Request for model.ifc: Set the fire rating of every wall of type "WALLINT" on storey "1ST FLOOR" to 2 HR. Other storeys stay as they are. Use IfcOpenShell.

First a look at what the model holds.

```python
import ifcopenshell
import ifcopenshell.util.element

model = ifcopenshell.open("model.ifc")
print(model.schema)
storey = next(s for s in model.by_type("IfcBuildingStorey") if s.Name == "1ST FLOOR")
walls = [e for e in ifcopenshell.util.element.get_decomposition(storey) if e.is_a("IfcWall")]
seen = {}
for e in walls:
    element_type = ifcopenshell.util.element.get_type(e)
    key = (element_type.Name if element_type != e and element_type else None, ifcopenshell.util.element.get_pset(e, "Pset_WallCommon", "FireRating"))
    seen[key] = seen.get(key, 0) + 1
for (name, value), count in sorted(seen.items(), key=str):
    print(count, "x", name, "|", value)
```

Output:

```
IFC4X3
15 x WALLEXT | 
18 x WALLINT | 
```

```python
import ifcopenshell
import ifcopenshell.api.pset
import ifcopenshell.util.element

model = ifcopenshell.open("model.ifc")

storey = next(s for s in model.by_type("IfcBuildingStorey") if s.Name == "1ST FLOOR")
walls = [e for e in ifcopenshell.util.element.get_decomposition(storey) if e.is_a("IfcWall")]

count = 0
for e in walls:
    element_type = ifcopenshell.util.element.get_type(e)
    if element_type in (None, e) or element_type.Name != "WALLINT":
        continue
    # add_pset returns the element's existing set when there is one.
    pset = ifcopenshell.api.pset.add_pset(model, product=e, name="Pset_WallCommon")
    ifcopenshell.api.pset.edit_pset(model, pset=pset, properties={"FireRating": "2 HR"})
    count += 1

print(count, "walls updated")

model.write("model_rev.ifc")
```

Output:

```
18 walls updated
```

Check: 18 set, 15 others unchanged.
